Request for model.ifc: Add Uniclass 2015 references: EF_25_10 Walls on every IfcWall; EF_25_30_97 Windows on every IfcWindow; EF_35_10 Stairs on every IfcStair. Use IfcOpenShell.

First a look at what the model holds.

```python
import ifcopenshell

model = ifcopenshell.open("model.ifc")
print(model.schema)
print("classifications:", [c.Name for c in model.by_type("IfcClassification")])
for ifc_class in ("IfcDoor", "IfcRoof", "IfcStair", "IfcWall", "IfcWindow"):
    print(ifc_class, len(model.by_type(ifc_class)))
```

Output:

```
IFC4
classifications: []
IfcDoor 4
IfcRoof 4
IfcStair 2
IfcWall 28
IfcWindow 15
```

```python
import ifcopenshell
import ifcopenshell.api.classification

model = ifcopenshell.open("model.ifc")

system = ifcopenshell.api.classification.add_classification(model, classification="Uniclass 2015")

codes = {
    "IfcWall": ("EF_25_10", "Walls"),
    "IfcWindow": ("EF_25_30_97", "Windows"),
    "IfcStair": ("EF_35_10", "Stairs"),
}
for ifc_class, (code, name) in codes.items():
    products = model.by_type(ifc_class)
    ifcopenshell.api.classification.add_reference(
        model, products=products, classification=system, identification=code, name=name
    )
    print(code, len(products))

model.write("model_updated.ifc")
```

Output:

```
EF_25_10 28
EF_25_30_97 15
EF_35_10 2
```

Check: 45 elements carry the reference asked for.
